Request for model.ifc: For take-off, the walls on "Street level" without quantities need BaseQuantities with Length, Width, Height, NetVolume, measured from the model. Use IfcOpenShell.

First a look at what the model holds.

```python
import ifcopenshell
import ifcopenshell.util.element
import ifcopenshell.util.unit

model = ifcopenshell.open("model.ifc")
print(model.schema)
for unit_type in ("LENGTHUNIT", "AREAUNIT", "VOLUMEUNIT"):
    print(unit_type, ifcopenshell.util.unit.calculate_unit_scale(model, unit_type))
storey = next(s for s in model.by_type("IfcBuildingStorey") if s.Name == "Street level")
walls = [e for e in ifcopenshell.util.element.get_decomposition(storey) if e.is_a("IfcWall")]
for e in sorted(walls, key=lambda e: e.id()):
    print(e.id(), e.is_a(), e.Name, list(ifcopenshell.util.element.get_psets(e, qtos_only=True)), sep=" | ")
```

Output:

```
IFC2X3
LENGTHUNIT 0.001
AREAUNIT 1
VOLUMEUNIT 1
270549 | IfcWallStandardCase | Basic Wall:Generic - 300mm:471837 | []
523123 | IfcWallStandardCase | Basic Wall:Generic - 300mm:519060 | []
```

```python
import ifcopenshell
import ifcopenshell.api.pset
import ifcopenshell.geom
import ifcopenshell.util.element
import ifcopenshell.util.shape
import ifcopenshell.util.unit

model = ifcopenshell.open("model.ifc")
unit_scale = ifcopenshell.util.unit.calculate_unit_scale(model)
volume_scale = ifcopenshell.util.unit.calculate_unit_scale(model, "VOLUMEUNIT")
settings = ifcopenshell.geom.settings()

storey = next(s for s in model.by_type("IfcBuildingStorey") if s.Name == "Street level")
walls = [e for e in ifcopenshell.util.element.get_decomposition(storey) if e.is_a("IfcWall")]

for e in sorted(walls, key=lambda e: e.id()):
    if ifcopenshell.util.element.get_psets(e, qtos_only=True, should_inherit=False):
        continue
    # Geometry comes back in metres, in the element's own axes.
    shape = ifcopenshell.geom.create_shape(settings, e)
    values = {
        "Length": ifcopenshell.util.shape.get_x(shape.geometry) / unit_scale,
        "Width": ifcopenshell.util.shape.get_y(shape.geometry) / unit_scale,
        "Height": ifcopenshell.util.shape.get_z(shape.geometry) / unit_scale,
        "NetVolume": ifcopenshell.util.shape.get_volume(shape.geometry) / volume_scale,
    }
    qto = ifcopenshell.api.pset.add_qto(model, product=e, name="BaseQuantities")
    ifcopenshell.api.pset.edit_qto(model, qto=qto, properties=values)
    print(e.id(), {k: round(v, 3) for k, v in values.items()})

model.write("model_v2.ifc")
```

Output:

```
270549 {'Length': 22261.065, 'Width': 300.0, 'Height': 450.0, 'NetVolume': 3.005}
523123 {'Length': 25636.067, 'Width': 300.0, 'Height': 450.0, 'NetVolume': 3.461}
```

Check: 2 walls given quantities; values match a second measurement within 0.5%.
